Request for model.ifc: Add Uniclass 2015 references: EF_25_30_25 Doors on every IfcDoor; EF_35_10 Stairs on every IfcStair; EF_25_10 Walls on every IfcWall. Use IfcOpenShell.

First a look at what the model holds.

```python
import ifcopenshell

model = ifcopenshell.open("model.ifc")
print(model.schema)
print("classifications:", [c.Name for c in model.by_type("IfcClassification")])
for ifc_class in ("IfcDoor", "IfcRoof", "IfcStair", "IfcWall", "IfcWindow"):
    print(ifc_class, len(model.by_type(ifc_class)))
```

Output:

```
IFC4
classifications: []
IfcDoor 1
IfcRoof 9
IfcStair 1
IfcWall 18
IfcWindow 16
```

```python
import ifcopenshell
import ifcopenshell.api.classification

model = ifcopenshell.open("model.ifc")

system = ifcopenshell.api.classification.add_classification(model, classification="Uniclass 2015")

codes = {
    "IfcDoor": ("EF_25_30_25", "Doors"),
    "IfcStair": ("EF_35_10", "Stairs"),
    "IfcWall": ("EF_25_10", "Walls"),
}
for ifc_class, (code, name) in codes.items():
    products = model.by_type(ifc_class)
    ifcopenshell.api.classification.add_reference(
        model, products=products, classification=system, identification=code, name=name
    )
    print(code, len(products))

model.write("model_edited.ifc")
```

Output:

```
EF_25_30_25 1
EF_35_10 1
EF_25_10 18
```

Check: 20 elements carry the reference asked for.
